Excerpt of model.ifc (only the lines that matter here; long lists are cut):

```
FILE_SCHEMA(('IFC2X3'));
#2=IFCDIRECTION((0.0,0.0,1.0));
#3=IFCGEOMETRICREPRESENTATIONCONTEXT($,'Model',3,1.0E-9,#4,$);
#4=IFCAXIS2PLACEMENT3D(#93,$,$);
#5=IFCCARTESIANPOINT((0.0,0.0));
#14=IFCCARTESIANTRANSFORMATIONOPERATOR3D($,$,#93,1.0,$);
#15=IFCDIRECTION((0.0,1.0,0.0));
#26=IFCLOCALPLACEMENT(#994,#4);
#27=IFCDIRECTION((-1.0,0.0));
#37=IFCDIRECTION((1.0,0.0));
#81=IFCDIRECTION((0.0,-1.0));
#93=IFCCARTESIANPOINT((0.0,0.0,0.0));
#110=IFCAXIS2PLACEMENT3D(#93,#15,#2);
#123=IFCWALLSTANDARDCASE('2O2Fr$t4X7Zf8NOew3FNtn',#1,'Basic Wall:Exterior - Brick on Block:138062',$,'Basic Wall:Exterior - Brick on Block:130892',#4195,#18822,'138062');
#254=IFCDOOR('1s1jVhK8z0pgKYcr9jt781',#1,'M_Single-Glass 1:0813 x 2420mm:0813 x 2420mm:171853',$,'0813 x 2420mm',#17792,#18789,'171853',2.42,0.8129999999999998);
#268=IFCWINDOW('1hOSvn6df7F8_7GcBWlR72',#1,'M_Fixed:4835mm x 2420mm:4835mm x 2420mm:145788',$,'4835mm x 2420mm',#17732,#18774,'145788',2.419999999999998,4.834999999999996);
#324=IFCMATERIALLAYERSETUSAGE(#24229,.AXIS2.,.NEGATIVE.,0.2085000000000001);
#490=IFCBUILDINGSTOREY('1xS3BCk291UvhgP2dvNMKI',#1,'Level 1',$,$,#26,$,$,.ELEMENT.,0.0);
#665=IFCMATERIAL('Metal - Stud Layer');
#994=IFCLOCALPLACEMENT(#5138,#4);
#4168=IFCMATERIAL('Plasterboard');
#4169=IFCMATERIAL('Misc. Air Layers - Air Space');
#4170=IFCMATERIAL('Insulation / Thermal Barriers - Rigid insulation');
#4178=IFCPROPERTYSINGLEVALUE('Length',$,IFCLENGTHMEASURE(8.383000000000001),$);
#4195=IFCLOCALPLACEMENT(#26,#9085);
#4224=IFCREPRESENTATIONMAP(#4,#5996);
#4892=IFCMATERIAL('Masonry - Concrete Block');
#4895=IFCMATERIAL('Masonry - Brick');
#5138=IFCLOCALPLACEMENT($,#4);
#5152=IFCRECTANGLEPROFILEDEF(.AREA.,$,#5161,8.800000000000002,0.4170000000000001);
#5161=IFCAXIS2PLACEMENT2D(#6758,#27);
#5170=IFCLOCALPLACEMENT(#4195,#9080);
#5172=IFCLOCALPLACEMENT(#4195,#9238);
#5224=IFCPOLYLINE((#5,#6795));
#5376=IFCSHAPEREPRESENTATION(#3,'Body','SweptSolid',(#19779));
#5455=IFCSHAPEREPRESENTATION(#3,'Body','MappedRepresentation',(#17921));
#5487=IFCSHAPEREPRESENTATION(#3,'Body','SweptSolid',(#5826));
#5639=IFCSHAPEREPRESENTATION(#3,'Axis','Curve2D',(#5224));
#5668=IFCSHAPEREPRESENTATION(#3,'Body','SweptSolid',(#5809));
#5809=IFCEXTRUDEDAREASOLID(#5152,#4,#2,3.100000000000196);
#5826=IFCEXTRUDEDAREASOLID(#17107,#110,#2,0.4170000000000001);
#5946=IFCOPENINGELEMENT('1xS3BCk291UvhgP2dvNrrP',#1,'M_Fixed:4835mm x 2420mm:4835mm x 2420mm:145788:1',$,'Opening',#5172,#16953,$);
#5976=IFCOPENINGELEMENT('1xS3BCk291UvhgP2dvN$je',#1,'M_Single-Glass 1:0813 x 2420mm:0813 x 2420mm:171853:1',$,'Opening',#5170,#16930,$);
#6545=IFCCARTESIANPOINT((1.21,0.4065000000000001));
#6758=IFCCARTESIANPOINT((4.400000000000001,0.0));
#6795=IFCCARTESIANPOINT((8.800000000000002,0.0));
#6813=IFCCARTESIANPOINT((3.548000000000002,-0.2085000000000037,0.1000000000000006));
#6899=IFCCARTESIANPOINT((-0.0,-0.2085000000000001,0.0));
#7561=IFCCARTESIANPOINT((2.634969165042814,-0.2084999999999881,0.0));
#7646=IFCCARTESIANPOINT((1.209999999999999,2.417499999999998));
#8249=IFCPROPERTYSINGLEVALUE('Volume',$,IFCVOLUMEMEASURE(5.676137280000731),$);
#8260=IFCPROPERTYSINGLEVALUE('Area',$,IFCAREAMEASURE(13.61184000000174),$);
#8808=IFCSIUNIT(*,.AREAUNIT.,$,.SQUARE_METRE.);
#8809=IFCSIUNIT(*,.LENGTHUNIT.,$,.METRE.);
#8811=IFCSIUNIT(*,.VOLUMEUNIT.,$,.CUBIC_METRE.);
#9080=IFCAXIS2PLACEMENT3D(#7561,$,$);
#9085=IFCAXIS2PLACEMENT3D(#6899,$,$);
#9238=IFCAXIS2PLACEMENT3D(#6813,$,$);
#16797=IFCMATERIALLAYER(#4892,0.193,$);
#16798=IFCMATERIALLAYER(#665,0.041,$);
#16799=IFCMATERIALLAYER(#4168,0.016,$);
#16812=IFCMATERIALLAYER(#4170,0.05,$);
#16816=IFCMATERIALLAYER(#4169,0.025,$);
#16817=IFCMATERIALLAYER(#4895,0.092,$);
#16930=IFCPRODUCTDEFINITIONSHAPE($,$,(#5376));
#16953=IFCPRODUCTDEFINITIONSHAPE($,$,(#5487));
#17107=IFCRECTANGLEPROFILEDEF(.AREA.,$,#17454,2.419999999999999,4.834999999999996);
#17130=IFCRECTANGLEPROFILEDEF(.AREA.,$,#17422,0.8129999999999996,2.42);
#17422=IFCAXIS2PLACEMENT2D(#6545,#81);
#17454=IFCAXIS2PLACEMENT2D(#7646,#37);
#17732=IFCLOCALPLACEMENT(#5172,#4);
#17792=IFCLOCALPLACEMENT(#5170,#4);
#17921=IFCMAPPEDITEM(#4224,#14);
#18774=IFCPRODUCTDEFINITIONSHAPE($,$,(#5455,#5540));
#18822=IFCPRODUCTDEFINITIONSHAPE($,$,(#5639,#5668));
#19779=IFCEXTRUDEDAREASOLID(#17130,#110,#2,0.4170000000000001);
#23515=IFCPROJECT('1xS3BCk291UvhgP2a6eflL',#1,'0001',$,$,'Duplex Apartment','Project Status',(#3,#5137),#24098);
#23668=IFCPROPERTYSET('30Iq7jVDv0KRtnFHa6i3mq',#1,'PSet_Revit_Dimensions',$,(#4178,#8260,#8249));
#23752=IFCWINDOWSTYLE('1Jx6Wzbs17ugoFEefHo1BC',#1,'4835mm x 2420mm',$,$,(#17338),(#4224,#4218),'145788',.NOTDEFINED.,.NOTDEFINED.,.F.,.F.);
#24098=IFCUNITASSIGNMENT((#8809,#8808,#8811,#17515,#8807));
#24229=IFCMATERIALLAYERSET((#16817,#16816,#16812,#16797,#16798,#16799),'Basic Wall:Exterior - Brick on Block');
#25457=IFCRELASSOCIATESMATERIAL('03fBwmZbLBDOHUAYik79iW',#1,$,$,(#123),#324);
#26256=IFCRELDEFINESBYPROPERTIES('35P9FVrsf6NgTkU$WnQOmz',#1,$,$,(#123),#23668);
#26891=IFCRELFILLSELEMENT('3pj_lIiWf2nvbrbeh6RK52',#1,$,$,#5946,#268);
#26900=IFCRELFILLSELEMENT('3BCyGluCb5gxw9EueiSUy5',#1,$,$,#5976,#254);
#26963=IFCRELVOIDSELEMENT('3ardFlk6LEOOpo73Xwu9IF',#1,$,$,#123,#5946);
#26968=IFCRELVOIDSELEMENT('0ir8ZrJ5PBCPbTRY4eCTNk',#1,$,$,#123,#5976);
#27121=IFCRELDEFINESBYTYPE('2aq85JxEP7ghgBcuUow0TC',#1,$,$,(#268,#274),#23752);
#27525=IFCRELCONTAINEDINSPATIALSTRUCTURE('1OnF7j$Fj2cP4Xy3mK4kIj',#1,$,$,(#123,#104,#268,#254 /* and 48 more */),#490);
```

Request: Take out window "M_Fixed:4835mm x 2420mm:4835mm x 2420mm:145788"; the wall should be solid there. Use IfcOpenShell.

```python
import ifcopenshell
import ifcopenshell.api.feature
import ifcopenshell.api.pset
import ifcopenshell.api.root
import ifcopenshell.geom
import ifcopenshell.util.element
import ifcopenshell.util.shape
import ifcopenshell.util.unit

model = ifcopenshell.open("model.ifc")
area_scale = ifcopenshell.util.unit.calculate_unit_scale(model, "AREAUNIT")
volume_scale = ifcopenshell.util.unit.calculate_unit_scale(model, "VOLUMEUNIT")
settings = ifcopenshell.geom.settings()


def volume(element):
    """Net volume in cubic metres, openings subtracted."""
    shape = ifcopenshell.geom.create_shape(settings, element)
    return ifcopenshell.util.shape.get_volume(shape.geometry)


window = model.by_id(268)
opening = window.FillsVoids[0].RelatingOpeningElement
wall = opening.VoidsElements[0].RelatingBuildingElement
before = volume(wall)

ifcopenshell.api.root.remove_product(model, product=window)
ifcopenshell.api.feature.remove_feature(model, feature=opening)

after = volume(wall)
thickness = 0.417  # wall thickness in metres

# Update the wall's stored quantities.
pset = model.by_id(ifcopenshell.util.element.get_pset(wall, "PSet_Revit_Dimensions", should_inherit=False)["id"])
ifcopenshell.api.pset.edit_pset(model, pset=pset, properties={
    "Area": model.create_entity("IfcAreaMeasure", after / thickness / area_scale),
    "Volume": model.create_entity("IfcVolumeMeasure", after / volume_scale),
})

print(f"wall volume {before:.3f} -> {after:.3f} m3")

model.write("model-out.ifc")
```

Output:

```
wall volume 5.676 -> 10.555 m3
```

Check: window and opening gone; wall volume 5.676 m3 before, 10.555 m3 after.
